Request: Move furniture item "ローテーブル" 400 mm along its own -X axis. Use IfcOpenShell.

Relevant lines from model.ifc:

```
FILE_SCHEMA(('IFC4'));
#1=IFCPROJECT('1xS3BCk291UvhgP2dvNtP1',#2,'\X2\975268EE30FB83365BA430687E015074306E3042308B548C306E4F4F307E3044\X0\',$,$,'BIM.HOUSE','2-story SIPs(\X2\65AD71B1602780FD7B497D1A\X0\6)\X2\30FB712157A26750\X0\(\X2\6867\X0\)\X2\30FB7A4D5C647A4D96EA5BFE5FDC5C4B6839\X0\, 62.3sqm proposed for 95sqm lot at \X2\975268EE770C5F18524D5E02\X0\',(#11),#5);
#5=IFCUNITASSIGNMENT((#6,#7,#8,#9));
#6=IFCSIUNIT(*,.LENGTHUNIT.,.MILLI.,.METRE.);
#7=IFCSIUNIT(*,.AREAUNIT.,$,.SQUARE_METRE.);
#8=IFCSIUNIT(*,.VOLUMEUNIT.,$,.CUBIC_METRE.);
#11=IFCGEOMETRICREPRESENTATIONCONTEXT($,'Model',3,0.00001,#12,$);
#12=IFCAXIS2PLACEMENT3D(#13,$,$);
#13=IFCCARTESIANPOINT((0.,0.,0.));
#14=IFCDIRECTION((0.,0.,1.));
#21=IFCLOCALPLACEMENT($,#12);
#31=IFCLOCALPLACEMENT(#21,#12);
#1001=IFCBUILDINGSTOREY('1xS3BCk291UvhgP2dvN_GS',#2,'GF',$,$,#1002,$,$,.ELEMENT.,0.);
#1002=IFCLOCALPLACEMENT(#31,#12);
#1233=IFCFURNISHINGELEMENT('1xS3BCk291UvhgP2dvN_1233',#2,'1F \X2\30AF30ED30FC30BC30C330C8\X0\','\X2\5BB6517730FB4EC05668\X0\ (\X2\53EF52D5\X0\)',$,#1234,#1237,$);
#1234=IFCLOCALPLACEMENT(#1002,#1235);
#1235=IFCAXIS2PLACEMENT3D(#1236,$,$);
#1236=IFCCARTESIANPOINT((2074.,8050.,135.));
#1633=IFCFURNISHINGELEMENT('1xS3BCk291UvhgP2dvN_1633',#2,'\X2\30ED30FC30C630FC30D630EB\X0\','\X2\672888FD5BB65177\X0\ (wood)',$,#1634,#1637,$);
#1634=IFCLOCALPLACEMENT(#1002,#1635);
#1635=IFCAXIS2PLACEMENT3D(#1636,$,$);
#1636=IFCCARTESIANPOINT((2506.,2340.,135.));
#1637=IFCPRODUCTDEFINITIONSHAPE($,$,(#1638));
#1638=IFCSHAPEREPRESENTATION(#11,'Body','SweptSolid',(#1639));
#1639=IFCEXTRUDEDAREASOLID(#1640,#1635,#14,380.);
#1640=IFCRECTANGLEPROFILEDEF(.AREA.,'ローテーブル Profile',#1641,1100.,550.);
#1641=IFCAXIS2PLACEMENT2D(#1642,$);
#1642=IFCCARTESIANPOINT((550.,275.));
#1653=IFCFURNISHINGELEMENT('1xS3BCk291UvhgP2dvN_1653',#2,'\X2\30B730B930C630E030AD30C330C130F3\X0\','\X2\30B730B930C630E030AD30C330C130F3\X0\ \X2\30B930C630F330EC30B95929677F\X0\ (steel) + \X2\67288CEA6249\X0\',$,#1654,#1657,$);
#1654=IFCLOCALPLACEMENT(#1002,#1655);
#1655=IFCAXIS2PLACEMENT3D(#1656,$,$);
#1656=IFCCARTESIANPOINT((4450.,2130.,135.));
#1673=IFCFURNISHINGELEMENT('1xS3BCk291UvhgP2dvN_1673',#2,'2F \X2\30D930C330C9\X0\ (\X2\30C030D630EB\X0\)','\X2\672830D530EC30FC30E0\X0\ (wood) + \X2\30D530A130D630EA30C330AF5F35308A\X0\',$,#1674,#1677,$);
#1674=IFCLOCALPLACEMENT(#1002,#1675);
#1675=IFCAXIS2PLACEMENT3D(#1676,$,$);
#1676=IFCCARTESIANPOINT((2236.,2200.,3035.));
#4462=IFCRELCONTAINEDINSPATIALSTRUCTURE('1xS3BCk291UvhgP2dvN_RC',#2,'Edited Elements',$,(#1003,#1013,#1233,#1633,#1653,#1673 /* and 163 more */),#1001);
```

```python
import ifcopenshell
import ifcopenshell.api.geometry
import ifcopenshell.util.placement

model = ifcopenshell.open("model.ifc")

item = model.by_guid("1xS3BCk291UvhgP2dvN_1633")
matrix = ifcopenshell.util.placement.get_local_placement(item.ObjectPlacement)
matrix[:3, 3] -= matrix[:3, 0] * 400.0
ifcopenshell.api.geometry.edit_object_placement(model, product=item, matrix=matrix, is_si=False)

print(ifcopenshell.util.placement.get_local_placement(item.ObjectPlacement).round(3) + 0.0)

model.write("model_rev.ifc")
```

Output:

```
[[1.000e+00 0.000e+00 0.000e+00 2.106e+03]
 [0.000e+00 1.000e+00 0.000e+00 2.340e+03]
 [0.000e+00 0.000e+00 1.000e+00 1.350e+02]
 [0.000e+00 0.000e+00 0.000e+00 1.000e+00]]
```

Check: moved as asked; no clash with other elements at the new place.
